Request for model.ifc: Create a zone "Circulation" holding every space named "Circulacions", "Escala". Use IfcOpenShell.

First a look at what the model holds.

```python
import ifcopenshell

model = ifcopenshell.open("model.ifc")
print(model.schema)
seen = {}
for space in model.by_type("IfcSpace"):
    seen[space.LongName] = seen.get(space.LongName, 0) + 1
for name, count in sorted(seen.items(), key=str):
    print(count, "x", name)
print("zones:", [z.Name for z in model.by_type("IfcZone")][:20])
```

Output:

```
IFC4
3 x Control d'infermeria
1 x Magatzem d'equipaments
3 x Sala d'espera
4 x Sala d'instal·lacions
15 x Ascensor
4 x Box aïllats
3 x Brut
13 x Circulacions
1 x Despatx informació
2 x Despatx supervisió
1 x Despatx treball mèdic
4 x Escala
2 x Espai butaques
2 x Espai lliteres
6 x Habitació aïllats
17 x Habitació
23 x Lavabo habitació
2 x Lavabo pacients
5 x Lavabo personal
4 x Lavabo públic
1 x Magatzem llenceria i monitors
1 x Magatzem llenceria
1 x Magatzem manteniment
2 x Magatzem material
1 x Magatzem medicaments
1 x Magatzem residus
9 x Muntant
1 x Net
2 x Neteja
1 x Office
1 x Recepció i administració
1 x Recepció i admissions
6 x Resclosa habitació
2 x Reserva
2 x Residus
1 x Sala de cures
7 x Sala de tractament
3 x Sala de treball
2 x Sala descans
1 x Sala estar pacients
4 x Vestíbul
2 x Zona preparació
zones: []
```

```python
import ifcopenshell
import ifcopenshell.api.group
import ifcopenshell.api.root

model = ifcopenshell.open("model.ifc")

names = {"Circulacions", "Escala"}
spaces = [s for s in model.by_type("IfcSpace") if s.LongName in names]

zone = ifcopenshell.api.root.create_entity(model, ifc_class="IfcZone", name="Circulation")
ifcopenshell.api.group.assign_group(model, products=spaces, group=zone)
print(len(spaces), "spaces in", zone.Name)

model.write("model_updated.ifc")
```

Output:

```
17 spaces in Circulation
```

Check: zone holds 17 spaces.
